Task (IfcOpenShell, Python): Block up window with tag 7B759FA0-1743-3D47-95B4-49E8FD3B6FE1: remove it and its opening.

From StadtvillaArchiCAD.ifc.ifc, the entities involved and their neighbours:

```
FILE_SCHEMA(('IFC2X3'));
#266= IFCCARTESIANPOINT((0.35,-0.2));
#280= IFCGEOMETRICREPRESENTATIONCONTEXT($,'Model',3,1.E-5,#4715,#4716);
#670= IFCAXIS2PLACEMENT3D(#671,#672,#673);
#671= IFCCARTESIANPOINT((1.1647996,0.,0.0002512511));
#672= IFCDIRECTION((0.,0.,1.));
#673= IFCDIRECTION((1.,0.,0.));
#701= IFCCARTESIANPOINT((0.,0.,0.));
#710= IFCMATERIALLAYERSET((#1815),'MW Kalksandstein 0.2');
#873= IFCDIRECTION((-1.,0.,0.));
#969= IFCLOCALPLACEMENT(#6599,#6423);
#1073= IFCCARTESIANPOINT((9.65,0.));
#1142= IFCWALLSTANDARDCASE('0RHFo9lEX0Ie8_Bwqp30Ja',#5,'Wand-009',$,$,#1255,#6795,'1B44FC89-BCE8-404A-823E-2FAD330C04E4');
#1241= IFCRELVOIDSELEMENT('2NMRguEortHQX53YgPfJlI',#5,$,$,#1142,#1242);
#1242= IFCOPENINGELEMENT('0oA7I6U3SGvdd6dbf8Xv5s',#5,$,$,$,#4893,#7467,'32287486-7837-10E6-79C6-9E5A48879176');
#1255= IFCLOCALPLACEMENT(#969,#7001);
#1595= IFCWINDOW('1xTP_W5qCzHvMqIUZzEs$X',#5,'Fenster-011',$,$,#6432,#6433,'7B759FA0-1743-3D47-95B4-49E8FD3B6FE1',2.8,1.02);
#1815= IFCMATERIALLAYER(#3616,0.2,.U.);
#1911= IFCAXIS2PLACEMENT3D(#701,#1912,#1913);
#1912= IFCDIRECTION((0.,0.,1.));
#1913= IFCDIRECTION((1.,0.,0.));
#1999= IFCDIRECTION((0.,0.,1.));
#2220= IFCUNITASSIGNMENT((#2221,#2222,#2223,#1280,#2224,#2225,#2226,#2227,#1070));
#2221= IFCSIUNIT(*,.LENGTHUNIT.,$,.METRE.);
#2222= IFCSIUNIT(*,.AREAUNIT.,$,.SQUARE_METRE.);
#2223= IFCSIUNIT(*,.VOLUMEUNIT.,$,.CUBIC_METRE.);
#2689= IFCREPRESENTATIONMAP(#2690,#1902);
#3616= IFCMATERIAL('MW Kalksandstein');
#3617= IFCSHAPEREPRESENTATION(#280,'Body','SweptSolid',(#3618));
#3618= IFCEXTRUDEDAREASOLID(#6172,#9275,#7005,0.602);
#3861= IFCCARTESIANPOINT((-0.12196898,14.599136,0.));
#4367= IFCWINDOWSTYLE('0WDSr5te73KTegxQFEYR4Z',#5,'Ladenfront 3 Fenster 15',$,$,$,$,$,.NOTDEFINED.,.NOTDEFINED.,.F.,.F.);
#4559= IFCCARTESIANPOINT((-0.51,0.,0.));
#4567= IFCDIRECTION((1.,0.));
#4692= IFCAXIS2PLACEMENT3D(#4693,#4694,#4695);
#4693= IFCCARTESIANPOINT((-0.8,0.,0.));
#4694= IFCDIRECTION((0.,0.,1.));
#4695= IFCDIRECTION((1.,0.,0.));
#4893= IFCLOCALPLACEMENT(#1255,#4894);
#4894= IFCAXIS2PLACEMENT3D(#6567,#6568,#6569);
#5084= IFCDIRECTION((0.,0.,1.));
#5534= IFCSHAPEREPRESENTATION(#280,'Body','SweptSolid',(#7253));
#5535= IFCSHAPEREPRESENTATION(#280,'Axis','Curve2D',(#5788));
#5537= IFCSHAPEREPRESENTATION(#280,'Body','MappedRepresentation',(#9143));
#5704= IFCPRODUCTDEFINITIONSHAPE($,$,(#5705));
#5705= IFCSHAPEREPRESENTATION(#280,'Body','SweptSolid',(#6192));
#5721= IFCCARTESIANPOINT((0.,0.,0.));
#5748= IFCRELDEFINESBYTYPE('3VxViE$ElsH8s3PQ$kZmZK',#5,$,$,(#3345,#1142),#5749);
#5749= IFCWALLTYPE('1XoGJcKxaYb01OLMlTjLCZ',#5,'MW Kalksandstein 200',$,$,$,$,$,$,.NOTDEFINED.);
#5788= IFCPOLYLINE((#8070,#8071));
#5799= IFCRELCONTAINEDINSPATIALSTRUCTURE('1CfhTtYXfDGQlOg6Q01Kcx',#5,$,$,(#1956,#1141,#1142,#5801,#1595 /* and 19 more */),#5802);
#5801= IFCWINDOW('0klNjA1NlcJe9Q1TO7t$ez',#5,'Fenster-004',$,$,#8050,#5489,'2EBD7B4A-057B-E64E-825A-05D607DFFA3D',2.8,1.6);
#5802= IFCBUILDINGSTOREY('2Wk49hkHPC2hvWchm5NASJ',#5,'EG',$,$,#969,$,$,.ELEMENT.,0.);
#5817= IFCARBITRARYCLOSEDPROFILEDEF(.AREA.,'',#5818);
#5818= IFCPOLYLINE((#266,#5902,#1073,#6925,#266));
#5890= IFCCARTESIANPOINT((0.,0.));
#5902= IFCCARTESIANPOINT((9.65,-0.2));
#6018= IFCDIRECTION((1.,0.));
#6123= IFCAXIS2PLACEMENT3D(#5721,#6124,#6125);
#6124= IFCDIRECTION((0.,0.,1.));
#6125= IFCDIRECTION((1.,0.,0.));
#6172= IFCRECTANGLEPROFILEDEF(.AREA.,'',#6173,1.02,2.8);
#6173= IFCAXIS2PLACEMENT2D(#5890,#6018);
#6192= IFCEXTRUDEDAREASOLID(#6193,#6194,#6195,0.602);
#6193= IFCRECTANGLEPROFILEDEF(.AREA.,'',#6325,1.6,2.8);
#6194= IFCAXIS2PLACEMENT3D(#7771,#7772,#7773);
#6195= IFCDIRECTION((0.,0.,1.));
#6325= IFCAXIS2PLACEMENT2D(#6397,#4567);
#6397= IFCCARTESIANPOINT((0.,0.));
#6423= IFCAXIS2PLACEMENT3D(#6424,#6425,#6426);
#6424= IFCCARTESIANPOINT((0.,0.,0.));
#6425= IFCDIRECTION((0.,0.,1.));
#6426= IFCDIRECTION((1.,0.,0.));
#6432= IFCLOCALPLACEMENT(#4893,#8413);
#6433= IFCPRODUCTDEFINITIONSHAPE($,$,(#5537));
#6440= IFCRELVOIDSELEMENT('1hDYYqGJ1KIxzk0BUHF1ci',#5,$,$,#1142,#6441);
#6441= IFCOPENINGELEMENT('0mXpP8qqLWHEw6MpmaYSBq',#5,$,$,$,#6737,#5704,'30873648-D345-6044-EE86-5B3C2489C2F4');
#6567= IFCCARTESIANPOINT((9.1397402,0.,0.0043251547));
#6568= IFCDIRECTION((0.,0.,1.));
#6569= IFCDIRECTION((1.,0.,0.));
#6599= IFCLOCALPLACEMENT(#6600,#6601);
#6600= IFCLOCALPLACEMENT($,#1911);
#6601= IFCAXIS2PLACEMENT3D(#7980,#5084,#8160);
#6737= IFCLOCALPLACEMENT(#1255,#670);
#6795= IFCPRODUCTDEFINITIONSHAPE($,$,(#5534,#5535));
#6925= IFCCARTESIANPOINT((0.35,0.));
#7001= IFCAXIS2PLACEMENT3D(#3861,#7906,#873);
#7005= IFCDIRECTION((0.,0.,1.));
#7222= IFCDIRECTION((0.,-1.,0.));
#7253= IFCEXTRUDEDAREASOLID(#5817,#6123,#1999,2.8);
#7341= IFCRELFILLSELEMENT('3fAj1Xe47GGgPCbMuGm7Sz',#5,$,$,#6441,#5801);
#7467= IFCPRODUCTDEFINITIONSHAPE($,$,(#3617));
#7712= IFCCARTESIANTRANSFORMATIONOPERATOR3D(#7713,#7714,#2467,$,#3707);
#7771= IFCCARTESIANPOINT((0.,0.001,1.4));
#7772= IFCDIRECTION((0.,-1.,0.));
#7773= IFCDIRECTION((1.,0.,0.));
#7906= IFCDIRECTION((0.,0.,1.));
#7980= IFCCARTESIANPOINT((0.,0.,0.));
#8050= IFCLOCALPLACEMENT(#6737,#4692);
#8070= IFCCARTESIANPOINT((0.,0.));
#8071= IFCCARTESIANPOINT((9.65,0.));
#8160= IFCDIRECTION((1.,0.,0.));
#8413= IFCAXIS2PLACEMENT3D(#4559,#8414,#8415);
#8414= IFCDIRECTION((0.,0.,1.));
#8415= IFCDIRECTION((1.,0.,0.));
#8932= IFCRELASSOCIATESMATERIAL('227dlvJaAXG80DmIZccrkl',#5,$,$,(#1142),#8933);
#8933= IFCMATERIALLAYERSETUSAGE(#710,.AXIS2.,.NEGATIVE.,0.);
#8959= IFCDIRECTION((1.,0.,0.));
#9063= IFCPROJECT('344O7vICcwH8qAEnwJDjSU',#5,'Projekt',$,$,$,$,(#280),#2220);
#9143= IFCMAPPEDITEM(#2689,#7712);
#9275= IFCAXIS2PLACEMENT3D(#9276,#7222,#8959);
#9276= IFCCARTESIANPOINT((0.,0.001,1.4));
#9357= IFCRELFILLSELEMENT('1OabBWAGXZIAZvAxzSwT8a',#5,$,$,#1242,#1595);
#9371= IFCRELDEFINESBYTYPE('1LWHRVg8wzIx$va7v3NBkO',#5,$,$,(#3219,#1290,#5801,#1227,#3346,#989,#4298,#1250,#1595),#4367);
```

```python
import ifcopenshell
import ifcopenshell.api.feature
import ifcopenshell.api.root
import ifcopenshell.geom
import ifcopenshell.util.shape

model = ifcopenshell.open("StadtvillaArchiCAD.ifc.ifc")
settings = ifcopenshell.geom.settings()


def volume(element):
    """Net volume in cubic metres, openings subtracted."""
    shape = ifcopenshell.geom.create_shape(settings, element)
    return ifcopenshell.util.shape.get_volume(shape.geometry)


window = model.by_guid("1xTP_W5qCzHvMqIUZzEs$X")
opening = window.FillsVoids[0].RelatingOpeningElement
wall = opening.VoidsElements[0].RelatingBuildingElement
before = volume(wall)

ifcopenshell.api.root.remove_product(model, product=window)
ifcopenshell.api.feature.remove_feature(model, feature=opening)

after = volume(wall)

print(f"wall volume {before:.3f} -> {after:.3f} m3")

model.write("StadtvillaArchiCAD.ifc_updated.ifc")
```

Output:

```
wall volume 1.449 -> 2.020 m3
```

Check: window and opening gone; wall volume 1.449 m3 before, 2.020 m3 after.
